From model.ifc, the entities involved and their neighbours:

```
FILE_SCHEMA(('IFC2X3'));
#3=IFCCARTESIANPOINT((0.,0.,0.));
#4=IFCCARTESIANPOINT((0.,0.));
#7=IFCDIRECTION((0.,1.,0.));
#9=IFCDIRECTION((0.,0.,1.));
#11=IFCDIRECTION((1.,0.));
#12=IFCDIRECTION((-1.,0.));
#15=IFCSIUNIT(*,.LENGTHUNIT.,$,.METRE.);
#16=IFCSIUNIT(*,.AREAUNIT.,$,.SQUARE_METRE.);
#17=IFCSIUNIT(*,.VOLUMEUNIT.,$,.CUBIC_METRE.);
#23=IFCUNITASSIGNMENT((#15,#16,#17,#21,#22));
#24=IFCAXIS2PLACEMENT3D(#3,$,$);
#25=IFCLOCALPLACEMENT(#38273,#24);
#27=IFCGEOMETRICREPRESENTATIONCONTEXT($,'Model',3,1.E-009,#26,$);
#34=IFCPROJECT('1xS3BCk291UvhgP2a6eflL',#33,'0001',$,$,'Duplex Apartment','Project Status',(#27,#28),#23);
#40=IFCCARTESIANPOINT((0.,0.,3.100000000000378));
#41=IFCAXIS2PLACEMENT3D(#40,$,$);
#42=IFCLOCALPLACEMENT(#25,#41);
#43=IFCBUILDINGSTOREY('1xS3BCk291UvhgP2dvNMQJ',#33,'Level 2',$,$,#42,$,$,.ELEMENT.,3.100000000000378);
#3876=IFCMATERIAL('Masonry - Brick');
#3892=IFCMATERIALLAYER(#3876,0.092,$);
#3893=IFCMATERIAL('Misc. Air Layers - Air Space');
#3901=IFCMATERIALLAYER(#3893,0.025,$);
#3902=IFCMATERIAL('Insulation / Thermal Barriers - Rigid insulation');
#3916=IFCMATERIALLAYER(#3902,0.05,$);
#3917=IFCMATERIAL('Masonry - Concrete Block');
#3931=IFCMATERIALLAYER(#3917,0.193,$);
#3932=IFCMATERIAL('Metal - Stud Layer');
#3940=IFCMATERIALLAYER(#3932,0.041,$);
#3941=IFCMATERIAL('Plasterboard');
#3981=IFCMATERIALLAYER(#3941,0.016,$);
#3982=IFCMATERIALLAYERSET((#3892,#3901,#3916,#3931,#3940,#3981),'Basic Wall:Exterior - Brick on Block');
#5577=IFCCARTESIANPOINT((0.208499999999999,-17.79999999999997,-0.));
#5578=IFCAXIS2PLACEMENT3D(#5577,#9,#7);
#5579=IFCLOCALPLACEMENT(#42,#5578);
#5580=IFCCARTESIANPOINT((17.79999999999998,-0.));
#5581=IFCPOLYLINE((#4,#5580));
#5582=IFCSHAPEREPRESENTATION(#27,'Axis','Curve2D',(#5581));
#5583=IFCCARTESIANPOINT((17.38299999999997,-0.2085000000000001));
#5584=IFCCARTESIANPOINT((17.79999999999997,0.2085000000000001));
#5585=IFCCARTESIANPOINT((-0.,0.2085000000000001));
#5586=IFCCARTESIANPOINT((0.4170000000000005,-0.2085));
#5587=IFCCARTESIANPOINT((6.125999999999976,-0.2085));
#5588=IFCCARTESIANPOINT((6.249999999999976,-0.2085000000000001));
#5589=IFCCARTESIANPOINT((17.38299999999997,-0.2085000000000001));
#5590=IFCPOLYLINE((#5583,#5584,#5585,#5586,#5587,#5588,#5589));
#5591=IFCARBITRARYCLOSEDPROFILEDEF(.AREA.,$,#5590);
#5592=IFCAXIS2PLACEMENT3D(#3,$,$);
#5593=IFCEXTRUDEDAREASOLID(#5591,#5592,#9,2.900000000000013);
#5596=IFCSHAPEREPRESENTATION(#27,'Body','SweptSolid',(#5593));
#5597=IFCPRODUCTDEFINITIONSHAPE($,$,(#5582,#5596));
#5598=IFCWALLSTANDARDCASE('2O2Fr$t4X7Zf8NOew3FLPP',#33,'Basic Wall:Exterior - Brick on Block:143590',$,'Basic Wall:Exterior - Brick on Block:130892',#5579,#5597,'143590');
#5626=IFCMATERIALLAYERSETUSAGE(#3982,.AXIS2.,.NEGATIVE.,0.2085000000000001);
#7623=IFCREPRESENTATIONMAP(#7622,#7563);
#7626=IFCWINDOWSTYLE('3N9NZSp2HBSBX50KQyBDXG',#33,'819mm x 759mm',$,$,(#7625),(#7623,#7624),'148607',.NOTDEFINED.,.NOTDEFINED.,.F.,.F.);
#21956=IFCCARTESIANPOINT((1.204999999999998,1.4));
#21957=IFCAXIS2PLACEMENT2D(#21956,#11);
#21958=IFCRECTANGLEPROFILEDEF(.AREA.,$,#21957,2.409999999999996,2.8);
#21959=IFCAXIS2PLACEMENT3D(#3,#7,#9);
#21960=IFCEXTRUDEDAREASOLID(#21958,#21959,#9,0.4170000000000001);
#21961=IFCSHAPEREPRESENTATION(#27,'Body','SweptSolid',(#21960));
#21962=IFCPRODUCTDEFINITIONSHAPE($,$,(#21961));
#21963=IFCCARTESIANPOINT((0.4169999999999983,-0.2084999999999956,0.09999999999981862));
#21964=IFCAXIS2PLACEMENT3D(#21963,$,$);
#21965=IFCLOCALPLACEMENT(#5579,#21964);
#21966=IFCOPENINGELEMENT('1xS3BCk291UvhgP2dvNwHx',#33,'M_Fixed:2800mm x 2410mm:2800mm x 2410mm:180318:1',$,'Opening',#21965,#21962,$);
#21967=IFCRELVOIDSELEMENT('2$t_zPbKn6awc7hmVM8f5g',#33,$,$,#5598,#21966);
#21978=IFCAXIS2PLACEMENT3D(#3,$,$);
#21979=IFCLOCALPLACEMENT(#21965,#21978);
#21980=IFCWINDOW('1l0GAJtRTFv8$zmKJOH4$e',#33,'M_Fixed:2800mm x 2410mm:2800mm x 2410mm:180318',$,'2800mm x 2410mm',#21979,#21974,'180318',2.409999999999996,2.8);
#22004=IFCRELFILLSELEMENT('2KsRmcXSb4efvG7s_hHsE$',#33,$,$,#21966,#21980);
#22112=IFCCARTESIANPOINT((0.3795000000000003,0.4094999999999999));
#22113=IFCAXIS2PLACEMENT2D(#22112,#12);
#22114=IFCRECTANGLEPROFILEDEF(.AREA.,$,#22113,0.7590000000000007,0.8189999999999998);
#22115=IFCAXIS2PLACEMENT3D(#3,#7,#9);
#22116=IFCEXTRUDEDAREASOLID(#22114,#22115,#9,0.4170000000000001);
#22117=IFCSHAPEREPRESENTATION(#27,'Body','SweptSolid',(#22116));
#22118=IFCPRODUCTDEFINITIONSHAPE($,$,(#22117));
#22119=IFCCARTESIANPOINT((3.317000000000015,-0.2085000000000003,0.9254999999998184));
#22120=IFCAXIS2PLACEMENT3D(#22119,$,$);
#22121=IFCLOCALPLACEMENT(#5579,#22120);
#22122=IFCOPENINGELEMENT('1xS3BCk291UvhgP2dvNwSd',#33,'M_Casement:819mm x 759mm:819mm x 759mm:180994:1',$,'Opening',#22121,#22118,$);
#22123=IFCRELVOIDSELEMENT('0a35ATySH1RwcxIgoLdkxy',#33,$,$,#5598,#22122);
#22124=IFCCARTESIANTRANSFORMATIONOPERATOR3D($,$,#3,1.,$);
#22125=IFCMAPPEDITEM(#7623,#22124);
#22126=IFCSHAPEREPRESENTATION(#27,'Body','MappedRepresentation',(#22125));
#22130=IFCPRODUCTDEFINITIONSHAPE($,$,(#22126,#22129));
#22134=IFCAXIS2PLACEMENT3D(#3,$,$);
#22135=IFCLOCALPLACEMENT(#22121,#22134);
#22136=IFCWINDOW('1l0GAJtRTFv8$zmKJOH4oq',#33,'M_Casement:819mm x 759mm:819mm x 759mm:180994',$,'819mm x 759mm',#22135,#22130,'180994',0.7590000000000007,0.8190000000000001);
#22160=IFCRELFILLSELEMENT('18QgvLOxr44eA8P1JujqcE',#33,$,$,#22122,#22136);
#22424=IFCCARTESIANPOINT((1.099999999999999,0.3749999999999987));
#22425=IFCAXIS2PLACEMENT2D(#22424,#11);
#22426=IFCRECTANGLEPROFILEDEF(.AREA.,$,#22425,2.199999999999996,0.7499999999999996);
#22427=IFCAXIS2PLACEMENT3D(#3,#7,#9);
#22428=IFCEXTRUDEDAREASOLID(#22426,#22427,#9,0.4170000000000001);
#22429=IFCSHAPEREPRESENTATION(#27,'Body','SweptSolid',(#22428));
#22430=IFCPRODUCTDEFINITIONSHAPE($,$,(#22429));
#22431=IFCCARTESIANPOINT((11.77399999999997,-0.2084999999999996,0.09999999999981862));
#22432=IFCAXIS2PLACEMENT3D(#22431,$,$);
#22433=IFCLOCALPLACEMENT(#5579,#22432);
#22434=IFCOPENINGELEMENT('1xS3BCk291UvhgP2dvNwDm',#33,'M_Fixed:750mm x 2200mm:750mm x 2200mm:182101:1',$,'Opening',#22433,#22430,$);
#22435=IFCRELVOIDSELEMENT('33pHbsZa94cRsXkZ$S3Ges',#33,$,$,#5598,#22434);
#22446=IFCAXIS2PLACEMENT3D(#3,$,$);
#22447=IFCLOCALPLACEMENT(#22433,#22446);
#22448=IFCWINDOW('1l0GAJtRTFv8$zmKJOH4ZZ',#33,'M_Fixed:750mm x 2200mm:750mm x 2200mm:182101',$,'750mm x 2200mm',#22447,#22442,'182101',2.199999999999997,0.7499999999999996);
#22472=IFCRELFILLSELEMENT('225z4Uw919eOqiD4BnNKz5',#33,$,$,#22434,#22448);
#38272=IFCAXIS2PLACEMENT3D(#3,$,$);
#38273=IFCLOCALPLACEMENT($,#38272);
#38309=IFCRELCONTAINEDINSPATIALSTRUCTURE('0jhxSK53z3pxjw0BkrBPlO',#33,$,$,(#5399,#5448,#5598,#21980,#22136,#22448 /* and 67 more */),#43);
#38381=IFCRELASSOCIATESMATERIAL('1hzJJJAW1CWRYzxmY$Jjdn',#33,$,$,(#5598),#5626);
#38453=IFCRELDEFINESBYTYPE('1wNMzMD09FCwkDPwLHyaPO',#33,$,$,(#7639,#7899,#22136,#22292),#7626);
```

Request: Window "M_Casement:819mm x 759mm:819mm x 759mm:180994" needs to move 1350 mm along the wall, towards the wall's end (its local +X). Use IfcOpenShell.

```python
import ifcopenshell
import ifcopenshell.api.geometry
import ifcopenshell.util.placement

model = ifcopenshell.open("model.ifc")

window = model.by_id(22136)
opening = window.FillsVoids[0].RelatingOpeningElement
wall = opening.VoidsElements[0].RelatingBuildingElement

wall_matrix = ifcopenshell.util.placement.get_local_placement(wall.ObjectPlacement)
shift = wall_matrix[:3, 0] * 1.35
before = ifcopenshell.util.placement.get_local_placement(window.ObjectPlacement)[:3, 3].copy()

# The window is placed relative to its opening, so it follows when the opening moves.
matrix = ifcopenshell.util.placement.get_local_placement(opening.ObjectPlacement)
matrix[:3, 3] += shift
ifcopenshell.api.geometry.edit_object_placement(
    model, product=opening, matrix=matrix, is_si=False, should_transform_children=True
)

after = ifcopenshell.util.placement.get_local_placement(window.ObjectPlacement)[:3, 3]
print("window moved by", (after - before).round(3) + 0.0)

model.write("model_v2.ifc")
```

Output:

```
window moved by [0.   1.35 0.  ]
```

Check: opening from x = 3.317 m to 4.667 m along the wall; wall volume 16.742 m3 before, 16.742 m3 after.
